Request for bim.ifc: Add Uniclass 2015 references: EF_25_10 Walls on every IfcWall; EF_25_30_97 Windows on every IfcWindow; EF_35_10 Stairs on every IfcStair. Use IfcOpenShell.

First a look at what the model holds.

```python
import ifcopenshell

model = ifcopenshell.open("bim.ifc")
print(model.schema)
print("classifications:", [c.Name for c in model.by_type("IfcClassification")])
for ifc_class in ("IfcDoor", "IfcRoof", "IfcStair", "IfcWall", "IfcWindow"):
    print(ifc_class, len(model.by_type(ifc_class)))
```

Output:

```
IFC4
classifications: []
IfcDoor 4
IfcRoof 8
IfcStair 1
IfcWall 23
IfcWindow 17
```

```python
import ifcopenshell
import ifcopenshell.api.classification

model = ifcopenshell.open("bim.ifc")

system = ifcopenshell.api.classification.add_classification(model, classification="Uniclass 2015")

codes = {
    "IfcWall": ("EF_25_10", "Walls"),
    "IfcWindow": ("EF_25_30_97", "Windows"),
    "IfcStair": ("EF_35_10", "Stairs"),
}
for ifc_class, (code, name) in codes.items():
    products = model.by_type(ifc_class)
    ifcopenshell.api.classification.add_reference(
        model, products=products, classification=system, identification=code, name=name
    )
    print(code, len(products))

model.write("bim-out.ifc")
```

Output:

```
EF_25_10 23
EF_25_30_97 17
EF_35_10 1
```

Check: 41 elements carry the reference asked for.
